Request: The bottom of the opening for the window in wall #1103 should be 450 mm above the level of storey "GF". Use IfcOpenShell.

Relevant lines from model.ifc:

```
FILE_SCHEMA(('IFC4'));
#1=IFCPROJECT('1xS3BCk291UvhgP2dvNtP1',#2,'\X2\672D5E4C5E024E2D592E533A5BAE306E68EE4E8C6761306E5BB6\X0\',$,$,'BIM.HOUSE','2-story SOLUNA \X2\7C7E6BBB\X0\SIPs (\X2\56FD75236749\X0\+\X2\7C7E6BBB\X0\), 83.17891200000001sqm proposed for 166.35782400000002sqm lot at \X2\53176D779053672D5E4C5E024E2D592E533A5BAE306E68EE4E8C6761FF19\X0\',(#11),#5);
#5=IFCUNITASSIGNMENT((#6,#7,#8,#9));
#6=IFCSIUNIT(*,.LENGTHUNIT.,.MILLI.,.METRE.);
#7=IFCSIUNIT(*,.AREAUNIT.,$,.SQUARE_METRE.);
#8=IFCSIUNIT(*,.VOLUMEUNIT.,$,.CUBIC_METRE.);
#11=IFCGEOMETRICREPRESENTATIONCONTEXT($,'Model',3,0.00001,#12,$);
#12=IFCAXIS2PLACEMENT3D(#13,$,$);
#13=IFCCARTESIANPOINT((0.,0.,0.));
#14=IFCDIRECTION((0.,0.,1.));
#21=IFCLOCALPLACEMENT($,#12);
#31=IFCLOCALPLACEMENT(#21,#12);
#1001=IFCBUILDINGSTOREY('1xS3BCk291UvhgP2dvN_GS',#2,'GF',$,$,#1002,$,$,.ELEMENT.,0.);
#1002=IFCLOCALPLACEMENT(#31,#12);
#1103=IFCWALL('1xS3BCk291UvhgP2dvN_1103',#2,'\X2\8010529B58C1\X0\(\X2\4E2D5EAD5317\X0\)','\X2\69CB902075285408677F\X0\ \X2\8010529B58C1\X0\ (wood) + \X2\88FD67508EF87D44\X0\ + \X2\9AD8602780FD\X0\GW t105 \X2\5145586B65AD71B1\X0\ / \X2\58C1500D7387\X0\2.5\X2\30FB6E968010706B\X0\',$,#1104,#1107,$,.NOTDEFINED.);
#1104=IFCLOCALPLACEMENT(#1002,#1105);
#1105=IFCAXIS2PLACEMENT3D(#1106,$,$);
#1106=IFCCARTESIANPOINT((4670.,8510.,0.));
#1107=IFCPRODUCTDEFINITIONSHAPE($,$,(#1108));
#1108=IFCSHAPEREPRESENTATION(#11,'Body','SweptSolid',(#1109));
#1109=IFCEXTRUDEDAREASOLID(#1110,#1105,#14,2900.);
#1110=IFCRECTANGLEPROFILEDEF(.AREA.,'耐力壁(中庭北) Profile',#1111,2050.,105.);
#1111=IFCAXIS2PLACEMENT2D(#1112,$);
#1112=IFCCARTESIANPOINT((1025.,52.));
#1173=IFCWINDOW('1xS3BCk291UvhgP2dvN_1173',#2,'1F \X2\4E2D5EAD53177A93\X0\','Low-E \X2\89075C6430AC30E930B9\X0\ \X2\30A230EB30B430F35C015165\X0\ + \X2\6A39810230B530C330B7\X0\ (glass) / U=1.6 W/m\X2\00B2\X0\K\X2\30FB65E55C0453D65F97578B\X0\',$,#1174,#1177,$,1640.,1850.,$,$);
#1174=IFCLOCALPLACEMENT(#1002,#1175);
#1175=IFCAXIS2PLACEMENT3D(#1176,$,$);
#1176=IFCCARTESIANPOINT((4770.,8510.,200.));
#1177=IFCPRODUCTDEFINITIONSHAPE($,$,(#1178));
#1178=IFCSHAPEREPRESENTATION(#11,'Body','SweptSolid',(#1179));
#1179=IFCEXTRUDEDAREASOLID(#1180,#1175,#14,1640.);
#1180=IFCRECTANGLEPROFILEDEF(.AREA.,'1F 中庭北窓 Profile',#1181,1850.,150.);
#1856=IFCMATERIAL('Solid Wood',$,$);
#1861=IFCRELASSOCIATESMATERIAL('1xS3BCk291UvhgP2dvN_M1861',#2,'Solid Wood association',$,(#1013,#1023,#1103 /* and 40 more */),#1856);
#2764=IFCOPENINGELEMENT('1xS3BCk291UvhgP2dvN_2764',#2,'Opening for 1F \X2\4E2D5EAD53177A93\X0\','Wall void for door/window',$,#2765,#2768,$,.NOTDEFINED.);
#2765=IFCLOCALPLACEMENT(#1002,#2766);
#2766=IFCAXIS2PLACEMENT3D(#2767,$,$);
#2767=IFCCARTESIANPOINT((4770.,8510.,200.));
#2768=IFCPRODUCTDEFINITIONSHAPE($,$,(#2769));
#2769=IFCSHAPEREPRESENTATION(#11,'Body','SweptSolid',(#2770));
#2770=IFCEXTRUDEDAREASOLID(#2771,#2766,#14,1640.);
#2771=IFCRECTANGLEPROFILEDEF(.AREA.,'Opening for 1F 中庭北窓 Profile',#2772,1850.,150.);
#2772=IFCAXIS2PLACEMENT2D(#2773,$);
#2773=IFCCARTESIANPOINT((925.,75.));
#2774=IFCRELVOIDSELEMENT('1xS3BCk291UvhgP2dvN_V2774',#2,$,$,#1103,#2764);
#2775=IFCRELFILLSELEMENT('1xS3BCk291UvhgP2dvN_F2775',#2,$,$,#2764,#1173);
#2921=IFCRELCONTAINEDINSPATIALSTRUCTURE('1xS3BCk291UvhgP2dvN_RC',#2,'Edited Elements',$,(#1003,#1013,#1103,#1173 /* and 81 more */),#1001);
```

```python
import numpy as np
import ifcopenshell
import ifcopenshell.api.geometry
import ifcopenshell.geom
import ifcopenshell.util.element
import ifcopenshell.util.placement
import ifcopenshell.util.shape
import ifcopenshell.util.unit

model = ifcopenshell.open("model.ifc")
unit_scale = ifcopenshell.util.unit.calculate_unit_scale(model)

window = model.by_guid("1xS3BCk291UvhgP2dvN_1173")
opening = window.FillsVoids[0].RelatingOpeningElement
storey = ifcopenshell.util.element.get_container(window, ifc_class="IfcBuildingStorey")
level = ifcopenshell.util.placement.get_local_placement(storey.ObjectPlacement)[2, 3]

# The opening's origin need not be at the sill, so measure its lowest point.
shape = ifcopenshell.geom.create_shape(ifcopenshell.geom.settings(), opening)
bottom = ifcopenshell.util.shape.get_shape_bottom_elevation(shape, shape.geometry) / unit_scale
dz = level + 450.0 - bottom

shift = np.array([0.0, 0.0, dz])
# The window is not placed relative to its opening, so move both.
for product in (opening, window):
    matrix = ifcopenshell.util.placement.get_local_placement(product.ObjectPlacement)
    matrix[:3, 3] += shift
    ifcopenshell.api.geometry.edit_object_placement(model, product=product, matrix=matrix, is_si=False)

print(f"moved by {dz * unit_scale:+.3f} m")

model.write("model_rev.ifc")
```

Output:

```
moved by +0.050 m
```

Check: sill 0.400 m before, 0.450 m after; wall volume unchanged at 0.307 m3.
